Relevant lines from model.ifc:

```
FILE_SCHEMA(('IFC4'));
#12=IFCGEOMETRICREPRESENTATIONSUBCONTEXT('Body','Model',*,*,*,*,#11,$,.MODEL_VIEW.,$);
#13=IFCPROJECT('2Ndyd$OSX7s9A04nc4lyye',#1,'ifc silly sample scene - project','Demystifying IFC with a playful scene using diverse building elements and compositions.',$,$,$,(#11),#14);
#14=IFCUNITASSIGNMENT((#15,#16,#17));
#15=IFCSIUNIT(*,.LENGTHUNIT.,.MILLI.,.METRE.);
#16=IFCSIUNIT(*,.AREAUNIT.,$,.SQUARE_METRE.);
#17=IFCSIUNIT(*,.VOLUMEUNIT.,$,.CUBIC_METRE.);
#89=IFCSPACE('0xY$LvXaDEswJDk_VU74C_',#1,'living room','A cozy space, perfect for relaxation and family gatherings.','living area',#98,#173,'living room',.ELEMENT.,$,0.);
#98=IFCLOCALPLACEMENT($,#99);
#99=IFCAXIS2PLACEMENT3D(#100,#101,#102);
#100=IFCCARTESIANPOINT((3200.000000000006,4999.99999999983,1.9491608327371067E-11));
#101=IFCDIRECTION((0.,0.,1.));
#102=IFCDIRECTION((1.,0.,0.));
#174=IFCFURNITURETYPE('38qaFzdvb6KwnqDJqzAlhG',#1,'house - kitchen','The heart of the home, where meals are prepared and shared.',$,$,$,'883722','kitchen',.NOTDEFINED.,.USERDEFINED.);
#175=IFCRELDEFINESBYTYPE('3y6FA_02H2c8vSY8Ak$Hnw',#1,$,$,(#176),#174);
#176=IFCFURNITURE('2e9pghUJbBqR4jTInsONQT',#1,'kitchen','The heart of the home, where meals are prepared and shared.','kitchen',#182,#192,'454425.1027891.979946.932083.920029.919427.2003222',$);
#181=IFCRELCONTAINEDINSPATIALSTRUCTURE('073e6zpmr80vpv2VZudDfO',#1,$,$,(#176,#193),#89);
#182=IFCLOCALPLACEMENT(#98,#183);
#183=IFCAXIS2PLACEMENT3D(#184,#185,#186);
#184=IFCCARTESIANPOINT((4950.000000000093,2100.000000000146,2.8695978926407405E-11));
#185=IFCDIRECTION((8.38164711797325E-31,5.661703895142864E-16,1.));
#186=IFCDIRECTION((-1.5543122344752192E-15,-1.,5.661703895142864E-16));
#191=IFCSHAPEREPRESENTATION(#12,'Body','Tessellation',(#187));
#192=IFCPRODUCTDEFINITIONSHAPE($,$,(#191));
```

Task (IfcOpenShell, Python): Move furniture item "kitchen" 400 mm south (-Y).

```python
import ifcopenshell
import ifcopenshell.api.geometry
import ifcopenshell.util.placement

model = ifcopenshell.open("model.ifc")

item = model.by_guid("2e9pghUJbBqR4jTInsONQT")
matrix = ifcopenshell.util.placement.get_local_placement(item.ObjectPlacement)
matrix[1, 3] -= 400.0
ifcopenshell.api.geometry.edit_object_placement(model, product=item, matrix=matrix, is_si=False)

print(ifcopenshell.util.placement.get_local_placement(item.ObjectPlacement).round(3) + 0.0)

model.write("model_edited.ifc")
```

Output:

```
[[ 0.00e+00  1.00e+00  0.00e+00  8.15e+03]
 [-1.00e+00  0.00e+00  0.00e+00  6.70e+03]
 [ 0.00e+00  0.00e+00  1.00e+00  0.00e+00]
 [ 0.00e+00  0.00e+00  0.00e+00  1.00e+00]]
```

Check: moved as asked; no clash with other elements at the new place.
